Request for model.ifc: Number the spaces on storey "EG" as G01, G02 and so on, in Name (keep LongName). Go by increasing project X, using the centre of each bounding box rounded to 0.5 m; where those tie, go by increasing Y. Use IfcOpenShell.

First a look at what the model holds.

```python
import ifcopenshell
import ifcopenshell.util.element
import ifcopenshell.util.placement

model = ifcopenshell.open("model.ifc")
print(model.schema)
storey = next(s for s in model.by_type("IfcBuildingStorey") if s.Name == "EG")
spaces = [e for e in ifcopenshell.util.element.get_decomposition(storey) if e.is_a("IfcSpace")]
for e in sorted(spaces, key=lambda e: e.id()):
    origin = ifcopenshell.util.placement.get_local_placement(e.ObjectPlacement)[:3, 3]
    print(e.id(), e.Name, e.LongName, origin.round(2) + 0.0, sep=" | ")
```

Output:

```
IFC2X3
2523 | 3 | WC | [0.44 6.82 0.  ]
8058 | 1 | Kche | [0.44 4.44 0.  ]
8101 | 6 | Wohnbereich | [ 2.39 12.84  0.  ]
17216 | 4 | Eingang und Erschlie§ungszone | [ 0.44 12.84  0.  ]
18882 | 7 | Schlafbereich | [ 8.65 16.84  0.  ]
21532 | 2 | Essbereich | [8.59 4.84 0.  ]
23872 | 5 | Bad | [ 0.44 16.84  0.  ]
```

```python
import ifcopenshell
import ifcopenshell.geom
import ifcopenshell.util.element
import ifcopenshell.util.shape

model = ifcopenshell.open("model.ifc")
settings = ifcopenshell.geom.settings()
settings.set("use-world-coords", True)


def centre(element):
    shape = ifcopenshell.geom.create_shape(settings, element)
    return ifcopenshell.util.shape.get_bbox_centroid(shape.geometry)


storey = next(s for s in model.by_type("IfcBuildingStorey") if s.Name == "EG")
spaces = [e for e in ifcopenshell.util.element.get_decomposition(storey) if e.is_a("IfcSpace")]

# Insertion points can sit at a corner or the storey origin, so sort by the geometry (in metres).
centres = {e: centre(e) for e in spaces}
spaces.sort(key=lambda e: (round(centres[e][0] / 0.5), centres[e][1]))

for i, e in enumerate(spaces, start=1):
    number = f"G{i:02d}"
    e.Name = number
    print(e.id(), number)

model.write("model_edited.ifc")
```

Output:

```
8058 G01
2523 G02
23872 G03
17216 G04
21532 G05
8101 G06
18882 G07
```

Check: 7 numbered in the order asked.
